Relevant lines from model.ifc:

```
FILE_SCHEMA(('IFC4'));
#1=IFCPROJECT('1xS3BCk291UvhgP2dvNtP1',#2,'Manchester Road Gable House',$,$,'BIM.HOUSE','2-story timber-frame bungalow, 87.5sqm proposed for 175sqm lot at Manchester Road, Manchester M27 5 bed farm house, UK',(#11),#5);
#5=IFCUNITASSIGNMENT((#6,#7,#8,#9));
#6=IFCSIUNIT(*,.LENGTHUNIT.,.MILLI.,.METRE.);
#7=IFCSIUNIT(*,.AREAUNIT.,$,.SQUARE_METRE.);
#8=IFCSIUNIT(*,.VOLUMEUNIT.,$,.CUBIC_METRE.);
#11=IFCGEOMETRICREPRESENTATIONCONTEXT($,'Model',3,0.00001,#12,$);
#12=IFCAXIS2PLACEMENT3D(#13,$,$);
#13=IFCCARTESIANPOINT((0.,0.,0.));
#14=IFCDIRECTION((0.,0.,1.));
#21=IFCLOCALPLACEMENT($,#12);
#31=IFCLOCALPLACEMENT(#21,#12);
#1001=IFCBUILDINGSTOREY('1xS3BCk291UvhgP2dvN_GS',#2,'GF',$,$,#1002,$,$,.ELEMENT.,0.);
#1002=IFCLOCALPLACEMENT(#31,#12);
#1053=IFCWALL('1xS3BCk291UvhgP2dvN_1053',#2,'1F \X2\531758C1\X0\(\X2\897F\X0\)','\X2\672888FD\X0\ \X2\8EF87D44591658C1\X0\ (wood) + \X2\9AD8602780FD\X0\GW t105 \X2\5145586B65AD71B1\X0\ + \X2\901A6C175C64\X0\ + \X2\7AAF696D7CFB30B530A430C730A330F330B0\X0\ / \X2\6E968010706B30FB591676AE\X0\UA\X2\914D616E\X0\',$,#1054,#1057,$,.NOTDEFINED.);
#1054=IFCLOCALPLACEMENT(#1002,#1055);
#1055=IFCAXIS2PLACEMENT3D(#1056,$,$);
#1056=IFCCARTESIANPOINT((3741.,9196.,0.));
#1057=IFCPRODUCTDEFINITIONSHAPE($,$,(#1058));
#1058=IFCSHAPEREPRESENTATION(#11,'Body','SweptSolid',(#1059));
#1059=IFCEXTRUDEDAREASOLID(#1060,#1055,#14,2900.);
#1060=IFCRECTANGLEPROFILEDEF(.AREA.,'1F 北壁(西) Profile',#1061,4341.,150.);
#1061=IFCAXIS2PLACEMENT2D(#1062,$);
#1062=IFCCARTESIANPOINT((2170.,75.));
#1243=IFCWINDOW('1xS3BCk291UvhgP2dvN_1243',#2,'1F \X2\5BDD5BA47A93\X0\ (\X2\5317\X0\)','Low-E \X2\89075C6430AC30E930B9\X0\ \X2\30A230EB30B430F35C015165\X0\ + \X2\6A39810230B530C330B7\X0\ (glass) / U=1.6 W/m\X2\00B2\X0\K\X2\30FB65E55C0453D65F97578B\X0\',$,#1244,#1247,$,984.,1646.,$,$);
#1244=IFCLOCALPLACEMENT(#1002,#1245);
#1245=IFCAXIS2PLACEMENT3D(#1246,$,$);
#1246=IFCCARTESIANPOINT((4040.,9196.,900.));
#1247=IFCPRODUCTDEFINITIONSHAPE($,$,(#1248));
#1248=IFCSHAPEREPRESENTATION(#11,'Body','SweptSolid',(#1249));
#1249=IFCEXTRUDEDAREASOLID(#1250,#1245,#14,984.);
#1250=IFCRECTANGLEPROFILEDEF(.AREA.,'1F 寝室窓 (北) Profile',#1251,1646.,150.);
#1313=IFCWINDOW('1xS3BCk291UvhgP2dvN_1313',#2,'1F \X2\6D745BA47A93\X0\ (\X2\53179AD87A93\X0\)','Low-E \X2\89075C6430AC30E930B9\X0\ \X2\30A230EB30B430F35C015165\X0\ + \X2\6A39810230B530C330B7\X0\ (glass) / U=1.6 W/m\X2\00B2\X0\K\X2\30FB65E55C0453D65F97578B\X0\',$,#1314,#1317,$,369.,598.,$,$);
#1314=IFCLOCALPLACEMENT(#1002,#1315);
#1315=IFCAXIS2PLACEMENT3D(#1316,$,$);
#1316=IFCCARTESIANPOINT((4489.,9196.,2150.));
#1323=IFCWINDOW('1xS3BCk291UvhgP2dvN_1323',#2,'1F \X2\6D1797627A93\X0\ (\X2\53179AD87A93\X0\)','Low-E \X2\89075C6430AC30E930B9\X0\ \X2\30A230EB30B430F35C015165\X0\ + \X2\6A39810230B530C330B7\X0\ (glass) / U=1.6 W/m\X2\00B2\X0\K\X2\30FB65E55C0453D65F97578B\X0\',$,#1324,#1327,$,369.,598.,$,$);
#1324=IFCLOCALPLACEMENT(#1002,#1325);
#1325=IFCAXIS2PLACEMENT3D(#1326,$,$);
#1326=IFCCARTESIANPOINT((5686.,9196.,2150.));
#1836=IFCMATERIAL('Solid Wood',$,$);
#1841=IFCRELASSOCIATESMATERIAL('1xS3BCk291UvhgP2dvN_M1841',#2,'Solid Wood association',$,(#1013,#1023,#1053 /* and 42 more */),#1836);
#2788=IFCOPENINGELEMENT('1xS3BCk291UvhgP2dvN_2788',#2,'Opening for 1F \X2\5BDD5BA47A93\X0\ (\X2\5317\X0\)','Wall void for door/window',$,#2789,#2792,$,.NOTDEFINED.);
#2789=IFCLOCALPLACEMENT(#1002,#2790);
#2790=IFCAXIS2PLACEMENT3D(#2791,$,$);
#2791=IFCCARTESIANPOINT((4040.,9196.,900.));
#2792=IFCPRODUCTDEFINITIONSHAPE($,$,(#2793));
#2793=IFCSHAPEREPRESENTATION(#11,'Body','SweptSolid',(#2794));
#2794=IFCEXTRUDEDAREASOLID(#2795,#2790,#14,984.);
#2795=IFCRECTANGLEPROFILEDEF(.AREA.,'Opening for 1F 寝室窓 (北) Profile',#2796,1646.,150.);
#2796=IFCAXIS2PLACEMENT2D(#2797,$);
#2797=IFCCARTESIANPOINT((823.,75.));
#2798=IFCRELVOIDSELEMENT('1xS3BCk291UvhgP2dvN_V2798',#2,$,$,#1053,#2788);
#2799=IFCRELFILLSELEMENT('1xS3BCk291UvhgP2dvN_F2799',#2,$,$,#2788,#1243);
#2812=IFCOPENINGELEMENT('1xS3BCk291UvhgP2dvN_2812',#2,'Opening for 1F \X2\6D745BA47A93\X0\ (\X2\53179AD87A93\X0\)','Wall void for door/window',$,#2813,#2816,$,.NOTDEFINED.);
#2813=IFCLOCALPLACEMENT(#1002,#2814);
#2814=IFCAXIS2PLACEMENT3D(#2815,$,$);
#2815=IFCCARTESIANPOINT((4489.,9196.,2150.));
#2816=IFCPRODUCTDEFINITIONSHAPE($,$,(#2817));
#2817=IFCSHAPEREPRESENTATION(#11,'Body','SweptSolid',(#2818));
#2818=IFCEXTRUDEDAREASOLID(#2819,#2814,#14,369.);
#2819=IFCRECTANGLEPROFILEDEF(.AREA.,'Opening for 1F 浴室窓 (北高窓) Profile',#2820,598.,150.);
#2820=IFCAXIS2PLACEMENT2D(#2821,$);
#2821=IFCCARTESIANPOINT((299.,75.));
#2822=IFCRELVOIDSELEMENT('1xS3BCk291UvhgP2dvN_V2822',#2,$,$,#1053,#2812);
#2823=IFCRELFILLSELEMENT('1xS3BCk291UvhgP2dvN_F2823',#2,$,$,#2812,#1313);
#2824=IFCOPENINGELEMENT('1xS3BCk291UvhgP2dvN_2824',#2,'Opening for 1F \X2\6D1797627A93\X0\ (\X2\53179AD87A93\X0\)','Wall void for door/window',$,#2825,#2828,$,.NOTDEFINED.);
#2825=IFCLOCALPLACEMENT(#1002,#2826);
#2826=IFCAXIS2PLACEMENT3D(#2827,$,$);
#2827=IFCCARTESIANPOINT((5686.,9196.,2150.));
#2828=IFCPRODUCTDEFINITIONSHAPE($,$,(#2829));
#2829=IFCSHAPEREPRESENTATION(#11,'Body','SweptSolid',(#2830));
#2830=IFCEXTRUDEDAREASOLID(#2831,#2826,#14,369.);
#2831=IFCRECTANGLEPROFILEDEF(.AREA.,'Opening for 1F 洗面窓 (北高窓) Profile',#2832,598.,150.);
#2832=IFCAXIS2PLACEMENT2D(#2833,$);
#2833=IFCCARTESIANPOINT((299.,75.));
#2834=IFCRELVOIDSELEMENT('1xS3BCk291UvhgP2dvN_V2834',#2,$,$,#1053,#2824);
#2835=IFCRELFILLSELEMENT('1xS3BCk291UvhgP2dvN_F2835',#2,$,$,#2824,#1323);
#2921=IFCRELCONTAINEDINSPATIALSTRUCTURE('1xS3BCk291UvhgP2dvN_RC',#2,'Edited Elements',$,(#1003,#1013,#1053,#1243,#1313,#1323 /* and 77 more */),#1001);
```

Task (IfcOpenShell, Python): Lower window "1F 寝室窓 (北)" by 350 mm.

```python
import numpy as np
import ifcopenshell
import ifcopenshell.api.geometry
import ifcopenshell.util.placement
import ifcopenshell.util.unit

model = ifcopenshell.open("model.ifc")
unit_scale = ifcopenshell.util.unit.calculate_unit_scale(model)

window = model.by_guid("1xS3BCk291UvhgP2dvN_1243")
opening = window.FillsVoids[0].RelatingOpeningElement
dz = -0.35 / unit_scale

shift = np.array([0.0, 0.0, dz])
# The window is not placed relative to its opening, so move both.
for product in (opening, window):
    matrix = ifcopenshell.util.placement.get_local_placement(product.ObjectPlacement)
    matrix[:3, 3] += shift
    ifcopenshell.api.geometry.edit_object_placement(model, product=product, matrix=matrix, is_si=False)

print(f"moved by {dz * unit_scale:+.3f} m")

model.write("model-out.ifc")
```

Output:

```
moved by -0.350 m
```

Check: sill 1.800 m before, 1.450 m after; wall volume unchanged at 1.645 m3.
